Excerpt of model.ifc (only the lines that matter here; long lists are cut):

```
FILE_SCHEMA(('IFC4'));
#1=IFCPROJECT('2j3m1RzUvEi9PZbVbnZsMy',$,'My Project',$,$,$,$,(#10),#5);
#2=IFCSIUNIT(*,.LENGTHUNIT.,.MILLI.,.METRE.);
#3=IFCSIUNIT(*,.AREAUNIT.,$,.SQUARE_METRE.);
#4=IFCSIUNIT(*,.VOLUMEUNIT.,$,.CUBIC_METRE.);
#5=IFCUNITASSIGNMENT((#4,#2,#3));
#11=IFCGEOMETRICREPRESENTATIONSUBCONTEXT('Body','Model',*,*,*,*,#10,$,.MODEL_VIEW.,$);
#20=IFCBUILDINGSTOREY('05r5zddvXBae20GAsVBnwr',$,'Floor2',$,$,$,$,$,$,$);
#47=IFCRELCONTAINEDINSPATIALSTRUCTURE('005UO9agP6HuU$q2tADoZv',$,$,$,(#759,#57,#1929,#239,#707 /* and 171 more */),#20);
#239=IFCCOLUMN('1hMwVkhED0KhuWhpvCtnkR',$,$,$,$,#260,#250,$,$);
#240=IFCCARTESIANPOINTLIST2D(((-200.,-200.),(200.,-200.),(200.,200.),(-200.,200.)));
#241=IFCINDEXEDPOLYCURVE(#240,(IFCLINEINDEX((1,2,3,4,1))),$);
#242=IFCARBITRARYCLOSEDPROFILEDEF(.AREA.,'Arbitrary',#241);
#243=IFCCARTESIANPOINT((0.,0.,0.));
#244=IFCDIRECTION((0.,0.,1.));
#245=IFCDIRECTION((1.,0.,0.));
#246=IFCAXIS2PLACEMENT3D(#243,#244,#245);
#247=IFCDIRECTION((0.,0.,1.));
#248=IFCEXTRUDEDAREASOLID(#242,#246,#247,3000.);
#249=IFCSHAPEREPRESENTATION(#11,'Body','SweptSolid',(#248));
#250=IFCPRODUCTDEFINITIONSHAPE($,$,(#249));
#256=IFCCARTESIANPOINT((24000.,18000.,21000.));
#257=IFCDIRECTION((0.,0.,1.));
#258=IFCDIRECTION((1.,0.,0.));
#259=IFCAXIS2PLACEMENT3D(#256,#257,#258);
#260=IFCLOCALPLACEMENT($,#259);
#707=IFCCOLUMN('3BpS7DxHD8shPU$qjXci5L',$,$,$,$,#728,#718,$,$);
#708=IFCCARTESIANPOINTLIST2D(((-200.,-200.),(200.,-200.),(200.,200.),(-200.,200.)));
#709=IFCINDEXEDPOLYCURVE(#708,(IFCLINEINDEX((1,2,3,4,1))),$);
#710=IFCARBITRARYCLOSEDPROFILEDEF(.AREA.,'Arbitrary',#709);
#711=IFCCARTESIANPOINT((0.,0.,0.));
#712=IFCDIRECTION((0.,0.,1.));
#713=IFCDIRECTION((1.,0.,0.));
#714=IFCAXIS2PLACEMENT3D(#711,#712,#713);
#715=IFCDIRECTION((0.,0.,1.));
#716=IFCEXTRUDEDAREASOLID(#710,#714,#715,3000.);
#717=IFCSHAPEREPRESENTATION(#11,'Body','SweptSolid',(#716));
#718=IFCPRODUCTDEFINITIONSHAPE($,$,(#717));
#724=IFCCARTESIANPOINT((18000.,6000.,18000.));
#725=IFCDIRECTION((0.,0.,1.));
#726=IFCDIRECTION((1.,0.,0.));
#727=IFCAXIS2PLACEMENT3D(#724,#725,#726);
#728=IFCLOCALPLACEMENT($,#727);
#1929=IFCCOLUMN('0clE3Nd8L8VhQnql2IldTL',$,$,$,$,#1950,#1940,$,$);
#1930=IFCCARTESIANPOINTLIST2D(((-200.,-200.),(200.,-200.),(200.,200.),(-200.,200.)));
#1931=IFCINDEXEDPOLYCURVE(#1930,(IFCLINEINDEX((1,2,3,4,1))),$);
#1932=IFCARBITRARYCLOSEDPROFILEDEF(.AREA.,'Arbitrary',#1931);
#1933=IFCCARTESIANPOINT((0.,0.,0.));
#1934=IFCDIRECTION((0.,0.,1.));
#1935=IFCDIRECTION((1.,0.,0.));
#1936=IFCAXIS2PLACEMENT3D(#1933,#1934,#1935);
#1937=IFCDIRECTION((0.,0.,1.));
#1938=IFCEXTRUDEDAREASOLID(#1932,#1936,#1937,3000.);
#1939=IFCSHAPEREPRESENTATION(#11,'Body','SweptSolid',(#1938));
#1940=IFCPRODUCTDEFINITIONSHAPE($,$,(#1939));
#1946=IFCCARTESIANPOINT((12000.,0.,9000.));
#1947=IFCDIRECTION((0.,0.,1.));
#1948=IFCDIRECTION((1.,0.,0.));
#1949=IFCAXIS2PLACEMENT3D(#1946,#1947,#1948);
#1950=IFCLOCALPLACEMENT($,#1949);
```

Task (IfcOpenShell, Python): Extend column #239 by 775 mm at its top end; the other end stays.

```python
import ifcopenshell
import ifcopenshell.util.representation
import ifcopenshell.util.unit

model = ifcopenshell.open("model.ifc")
unit_scale = ifcopenshell.util.unit.calculate_unit_scale(model)

member = model.by_guid("1hMwVkhED0KhuWhpvCtnkR")
change = 0.775 / unit_scale

# The extrusion runs towards the end named, so only its depth changes.
body = ifcopenshell.util.representation.get_representation(member, "Model", "Body")
solid = body.Items[0]
old_length = solid.Depth
solid.Depth += change

print(f"length {old_length:g} -> {solid.Depth:g}")

model.write("model_rev.ifc")
```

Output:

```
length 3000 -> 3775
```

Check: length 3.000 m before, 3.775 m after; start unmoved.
